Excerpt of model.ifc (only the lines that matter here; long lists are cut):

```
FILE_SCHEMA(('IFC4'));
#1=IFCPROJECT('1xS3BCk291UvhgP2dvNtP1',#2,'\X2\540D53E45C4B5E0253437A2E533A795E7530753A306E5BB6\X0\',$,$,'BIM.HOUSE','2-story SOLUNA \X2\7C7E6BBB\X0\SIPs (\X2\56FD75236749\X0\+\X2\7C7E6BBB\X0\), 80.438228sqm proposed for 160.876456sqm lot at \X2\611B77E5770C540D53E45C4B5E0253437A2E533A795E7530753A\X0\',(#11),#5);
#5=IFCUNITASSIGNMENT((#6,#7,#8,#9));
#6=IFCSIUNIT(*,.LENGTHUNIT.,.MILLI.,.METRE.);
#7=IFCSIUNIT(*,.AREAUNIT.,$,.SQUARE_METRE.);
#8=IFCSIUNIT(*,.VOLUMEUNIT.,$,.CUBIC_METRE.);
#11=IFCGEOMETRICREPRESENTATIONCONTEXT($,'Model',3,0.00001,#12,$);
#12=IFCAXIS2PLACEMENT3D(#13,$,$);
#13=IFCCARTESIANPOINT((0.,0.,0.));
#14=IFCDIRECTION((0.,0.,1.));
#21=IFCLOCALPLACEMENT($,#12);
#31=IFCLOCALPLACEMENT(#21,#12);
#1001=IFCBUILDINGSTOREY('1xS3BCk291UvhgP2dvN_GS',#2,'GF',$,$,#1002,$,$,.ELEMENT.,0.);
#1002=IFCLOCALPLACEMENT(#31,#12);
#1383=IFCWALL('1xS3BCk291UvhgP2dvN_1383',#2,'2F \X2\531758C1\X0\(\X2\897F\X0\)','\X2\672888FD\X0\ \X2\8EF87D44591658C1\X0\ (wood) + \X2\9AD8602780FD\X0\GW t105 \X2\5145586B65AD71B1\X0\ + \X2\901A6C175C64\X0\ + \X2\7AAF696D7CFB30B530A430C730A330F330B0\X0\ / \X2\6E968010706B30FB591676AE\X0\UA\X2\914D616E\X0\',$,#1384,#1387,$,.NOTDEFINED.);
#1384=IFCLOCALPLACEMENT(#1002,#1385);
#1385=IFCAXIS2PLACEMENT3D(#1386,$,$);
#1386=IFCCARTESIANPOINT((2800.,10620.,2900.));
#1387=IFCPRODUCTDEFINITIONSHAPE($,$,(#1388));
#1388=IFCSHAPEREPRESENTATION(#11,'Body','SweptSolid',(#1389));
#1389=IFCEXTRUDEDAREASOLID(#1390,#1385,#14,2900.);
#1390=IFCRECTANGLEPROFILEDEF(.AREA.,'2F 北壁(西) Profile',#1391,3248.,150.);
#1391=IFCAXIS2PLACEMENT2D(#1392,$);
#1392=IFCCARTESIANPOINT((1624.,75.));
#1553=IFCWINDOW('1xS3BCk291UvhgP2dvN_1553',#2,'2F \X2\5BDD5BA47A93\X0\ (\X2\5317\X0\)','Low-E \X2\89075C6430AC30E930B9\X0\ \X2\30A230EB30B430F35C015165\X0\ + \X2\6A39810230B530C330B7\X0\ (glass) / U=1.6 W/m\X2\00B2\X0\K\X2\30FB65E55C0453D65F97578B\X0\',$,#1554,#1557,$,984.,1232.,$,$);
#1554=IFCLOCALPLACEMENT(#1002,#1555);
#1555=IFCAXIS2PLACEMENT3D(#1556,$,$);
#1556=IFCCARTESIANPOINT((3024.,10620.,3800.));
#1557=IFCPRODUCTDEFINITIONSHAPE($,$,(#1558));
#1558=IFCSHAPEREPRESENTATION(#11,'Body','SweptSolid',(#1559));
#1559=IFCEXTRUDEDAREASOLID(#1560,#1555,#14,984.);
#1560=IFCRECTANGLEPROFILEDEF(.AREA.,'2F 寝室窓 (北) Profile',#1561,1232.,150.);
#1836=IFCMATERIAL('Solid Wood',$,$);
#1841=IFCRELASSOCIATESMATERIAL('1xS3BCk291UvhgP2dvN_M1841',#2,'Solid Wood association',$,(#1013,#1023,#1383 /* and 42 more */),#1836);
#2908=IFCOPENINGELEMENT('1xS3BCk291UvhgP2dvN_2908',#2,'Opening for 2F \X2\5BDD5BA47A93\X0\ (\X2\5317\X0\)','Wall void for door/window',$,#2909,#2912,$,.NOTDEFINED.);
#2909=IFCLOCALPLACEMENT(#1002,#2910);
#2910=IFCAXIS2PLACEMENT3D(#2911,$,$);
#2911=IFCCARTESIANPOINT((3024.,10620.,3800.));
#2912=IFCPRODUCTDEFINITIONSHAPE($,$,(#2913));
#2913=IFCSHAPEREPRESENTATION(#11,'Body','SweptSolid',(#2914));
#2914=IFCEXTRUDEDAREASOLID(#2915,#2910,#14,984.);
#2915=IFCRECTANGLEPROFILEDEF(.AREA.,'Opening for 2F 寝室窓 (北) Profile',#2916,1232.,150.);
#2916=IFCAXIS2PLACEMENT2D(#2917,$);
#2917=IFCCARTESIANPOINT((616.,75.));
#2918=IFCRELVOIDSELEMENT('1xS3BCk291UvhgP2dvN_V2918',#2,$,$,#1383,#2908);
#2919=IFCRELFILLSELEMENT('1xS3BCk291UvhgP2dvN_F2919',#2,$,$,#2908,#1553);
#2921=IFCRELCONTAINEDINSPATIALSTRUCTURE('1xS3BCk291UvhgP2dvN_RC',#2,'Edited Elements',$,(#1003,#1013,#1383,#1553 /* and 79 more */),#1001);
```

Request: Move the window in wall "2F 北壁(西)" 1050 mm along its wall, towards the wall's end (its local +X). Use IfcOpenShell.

```python
import ifcopenshell
import ifcopenshell.api.geometry
import ifcopenshell.util.placement
import ifcopenshell.util.unit

model = ifcopenshell.open("model.ifc")
unit_scale = ifcopenshell.util.unit.calculate_unit_scale(model)

window = model.by_guid("1xS3BCk291UvhgP2dvN_1553")
opening = window.FillsVoids[0].RelatingOpeningElement
wall = opening.VoidsElements[0].RelatingBuildingElement

wall_matrix = ifcopenshell.util.placement.get_local_placement(wall.ObjectPlacement)
shift = wall_matrix[:3, 0] * 1.05 / unit_scale
before = ifcopenshell.util.placement.get_local_placement(window.ObjectPlacement)[:3, 3].copy()

# The window is not placed relative to its opening, so move both.
for product in (opening, window):
    matrix = ifcopenshell.util.placement.get_local_placement(product.ObjectPlacement)
    matrix[:3, 3] += shift
    ifcopenshell.api.geometry.edit_object_placement(model, product=product, matrix=matrix, is_si=False)

after = ifcopenshell.util.placement.get_local_placement(window.ObjectPlacement)[:3, 3]
print("window moved by", (after - before).round(3) + 0.0)

model.write("model_v2.ifc")
```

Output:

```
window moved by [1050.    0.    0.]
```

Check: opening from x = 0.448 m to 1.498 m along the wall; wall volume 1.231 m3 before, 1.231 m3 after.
